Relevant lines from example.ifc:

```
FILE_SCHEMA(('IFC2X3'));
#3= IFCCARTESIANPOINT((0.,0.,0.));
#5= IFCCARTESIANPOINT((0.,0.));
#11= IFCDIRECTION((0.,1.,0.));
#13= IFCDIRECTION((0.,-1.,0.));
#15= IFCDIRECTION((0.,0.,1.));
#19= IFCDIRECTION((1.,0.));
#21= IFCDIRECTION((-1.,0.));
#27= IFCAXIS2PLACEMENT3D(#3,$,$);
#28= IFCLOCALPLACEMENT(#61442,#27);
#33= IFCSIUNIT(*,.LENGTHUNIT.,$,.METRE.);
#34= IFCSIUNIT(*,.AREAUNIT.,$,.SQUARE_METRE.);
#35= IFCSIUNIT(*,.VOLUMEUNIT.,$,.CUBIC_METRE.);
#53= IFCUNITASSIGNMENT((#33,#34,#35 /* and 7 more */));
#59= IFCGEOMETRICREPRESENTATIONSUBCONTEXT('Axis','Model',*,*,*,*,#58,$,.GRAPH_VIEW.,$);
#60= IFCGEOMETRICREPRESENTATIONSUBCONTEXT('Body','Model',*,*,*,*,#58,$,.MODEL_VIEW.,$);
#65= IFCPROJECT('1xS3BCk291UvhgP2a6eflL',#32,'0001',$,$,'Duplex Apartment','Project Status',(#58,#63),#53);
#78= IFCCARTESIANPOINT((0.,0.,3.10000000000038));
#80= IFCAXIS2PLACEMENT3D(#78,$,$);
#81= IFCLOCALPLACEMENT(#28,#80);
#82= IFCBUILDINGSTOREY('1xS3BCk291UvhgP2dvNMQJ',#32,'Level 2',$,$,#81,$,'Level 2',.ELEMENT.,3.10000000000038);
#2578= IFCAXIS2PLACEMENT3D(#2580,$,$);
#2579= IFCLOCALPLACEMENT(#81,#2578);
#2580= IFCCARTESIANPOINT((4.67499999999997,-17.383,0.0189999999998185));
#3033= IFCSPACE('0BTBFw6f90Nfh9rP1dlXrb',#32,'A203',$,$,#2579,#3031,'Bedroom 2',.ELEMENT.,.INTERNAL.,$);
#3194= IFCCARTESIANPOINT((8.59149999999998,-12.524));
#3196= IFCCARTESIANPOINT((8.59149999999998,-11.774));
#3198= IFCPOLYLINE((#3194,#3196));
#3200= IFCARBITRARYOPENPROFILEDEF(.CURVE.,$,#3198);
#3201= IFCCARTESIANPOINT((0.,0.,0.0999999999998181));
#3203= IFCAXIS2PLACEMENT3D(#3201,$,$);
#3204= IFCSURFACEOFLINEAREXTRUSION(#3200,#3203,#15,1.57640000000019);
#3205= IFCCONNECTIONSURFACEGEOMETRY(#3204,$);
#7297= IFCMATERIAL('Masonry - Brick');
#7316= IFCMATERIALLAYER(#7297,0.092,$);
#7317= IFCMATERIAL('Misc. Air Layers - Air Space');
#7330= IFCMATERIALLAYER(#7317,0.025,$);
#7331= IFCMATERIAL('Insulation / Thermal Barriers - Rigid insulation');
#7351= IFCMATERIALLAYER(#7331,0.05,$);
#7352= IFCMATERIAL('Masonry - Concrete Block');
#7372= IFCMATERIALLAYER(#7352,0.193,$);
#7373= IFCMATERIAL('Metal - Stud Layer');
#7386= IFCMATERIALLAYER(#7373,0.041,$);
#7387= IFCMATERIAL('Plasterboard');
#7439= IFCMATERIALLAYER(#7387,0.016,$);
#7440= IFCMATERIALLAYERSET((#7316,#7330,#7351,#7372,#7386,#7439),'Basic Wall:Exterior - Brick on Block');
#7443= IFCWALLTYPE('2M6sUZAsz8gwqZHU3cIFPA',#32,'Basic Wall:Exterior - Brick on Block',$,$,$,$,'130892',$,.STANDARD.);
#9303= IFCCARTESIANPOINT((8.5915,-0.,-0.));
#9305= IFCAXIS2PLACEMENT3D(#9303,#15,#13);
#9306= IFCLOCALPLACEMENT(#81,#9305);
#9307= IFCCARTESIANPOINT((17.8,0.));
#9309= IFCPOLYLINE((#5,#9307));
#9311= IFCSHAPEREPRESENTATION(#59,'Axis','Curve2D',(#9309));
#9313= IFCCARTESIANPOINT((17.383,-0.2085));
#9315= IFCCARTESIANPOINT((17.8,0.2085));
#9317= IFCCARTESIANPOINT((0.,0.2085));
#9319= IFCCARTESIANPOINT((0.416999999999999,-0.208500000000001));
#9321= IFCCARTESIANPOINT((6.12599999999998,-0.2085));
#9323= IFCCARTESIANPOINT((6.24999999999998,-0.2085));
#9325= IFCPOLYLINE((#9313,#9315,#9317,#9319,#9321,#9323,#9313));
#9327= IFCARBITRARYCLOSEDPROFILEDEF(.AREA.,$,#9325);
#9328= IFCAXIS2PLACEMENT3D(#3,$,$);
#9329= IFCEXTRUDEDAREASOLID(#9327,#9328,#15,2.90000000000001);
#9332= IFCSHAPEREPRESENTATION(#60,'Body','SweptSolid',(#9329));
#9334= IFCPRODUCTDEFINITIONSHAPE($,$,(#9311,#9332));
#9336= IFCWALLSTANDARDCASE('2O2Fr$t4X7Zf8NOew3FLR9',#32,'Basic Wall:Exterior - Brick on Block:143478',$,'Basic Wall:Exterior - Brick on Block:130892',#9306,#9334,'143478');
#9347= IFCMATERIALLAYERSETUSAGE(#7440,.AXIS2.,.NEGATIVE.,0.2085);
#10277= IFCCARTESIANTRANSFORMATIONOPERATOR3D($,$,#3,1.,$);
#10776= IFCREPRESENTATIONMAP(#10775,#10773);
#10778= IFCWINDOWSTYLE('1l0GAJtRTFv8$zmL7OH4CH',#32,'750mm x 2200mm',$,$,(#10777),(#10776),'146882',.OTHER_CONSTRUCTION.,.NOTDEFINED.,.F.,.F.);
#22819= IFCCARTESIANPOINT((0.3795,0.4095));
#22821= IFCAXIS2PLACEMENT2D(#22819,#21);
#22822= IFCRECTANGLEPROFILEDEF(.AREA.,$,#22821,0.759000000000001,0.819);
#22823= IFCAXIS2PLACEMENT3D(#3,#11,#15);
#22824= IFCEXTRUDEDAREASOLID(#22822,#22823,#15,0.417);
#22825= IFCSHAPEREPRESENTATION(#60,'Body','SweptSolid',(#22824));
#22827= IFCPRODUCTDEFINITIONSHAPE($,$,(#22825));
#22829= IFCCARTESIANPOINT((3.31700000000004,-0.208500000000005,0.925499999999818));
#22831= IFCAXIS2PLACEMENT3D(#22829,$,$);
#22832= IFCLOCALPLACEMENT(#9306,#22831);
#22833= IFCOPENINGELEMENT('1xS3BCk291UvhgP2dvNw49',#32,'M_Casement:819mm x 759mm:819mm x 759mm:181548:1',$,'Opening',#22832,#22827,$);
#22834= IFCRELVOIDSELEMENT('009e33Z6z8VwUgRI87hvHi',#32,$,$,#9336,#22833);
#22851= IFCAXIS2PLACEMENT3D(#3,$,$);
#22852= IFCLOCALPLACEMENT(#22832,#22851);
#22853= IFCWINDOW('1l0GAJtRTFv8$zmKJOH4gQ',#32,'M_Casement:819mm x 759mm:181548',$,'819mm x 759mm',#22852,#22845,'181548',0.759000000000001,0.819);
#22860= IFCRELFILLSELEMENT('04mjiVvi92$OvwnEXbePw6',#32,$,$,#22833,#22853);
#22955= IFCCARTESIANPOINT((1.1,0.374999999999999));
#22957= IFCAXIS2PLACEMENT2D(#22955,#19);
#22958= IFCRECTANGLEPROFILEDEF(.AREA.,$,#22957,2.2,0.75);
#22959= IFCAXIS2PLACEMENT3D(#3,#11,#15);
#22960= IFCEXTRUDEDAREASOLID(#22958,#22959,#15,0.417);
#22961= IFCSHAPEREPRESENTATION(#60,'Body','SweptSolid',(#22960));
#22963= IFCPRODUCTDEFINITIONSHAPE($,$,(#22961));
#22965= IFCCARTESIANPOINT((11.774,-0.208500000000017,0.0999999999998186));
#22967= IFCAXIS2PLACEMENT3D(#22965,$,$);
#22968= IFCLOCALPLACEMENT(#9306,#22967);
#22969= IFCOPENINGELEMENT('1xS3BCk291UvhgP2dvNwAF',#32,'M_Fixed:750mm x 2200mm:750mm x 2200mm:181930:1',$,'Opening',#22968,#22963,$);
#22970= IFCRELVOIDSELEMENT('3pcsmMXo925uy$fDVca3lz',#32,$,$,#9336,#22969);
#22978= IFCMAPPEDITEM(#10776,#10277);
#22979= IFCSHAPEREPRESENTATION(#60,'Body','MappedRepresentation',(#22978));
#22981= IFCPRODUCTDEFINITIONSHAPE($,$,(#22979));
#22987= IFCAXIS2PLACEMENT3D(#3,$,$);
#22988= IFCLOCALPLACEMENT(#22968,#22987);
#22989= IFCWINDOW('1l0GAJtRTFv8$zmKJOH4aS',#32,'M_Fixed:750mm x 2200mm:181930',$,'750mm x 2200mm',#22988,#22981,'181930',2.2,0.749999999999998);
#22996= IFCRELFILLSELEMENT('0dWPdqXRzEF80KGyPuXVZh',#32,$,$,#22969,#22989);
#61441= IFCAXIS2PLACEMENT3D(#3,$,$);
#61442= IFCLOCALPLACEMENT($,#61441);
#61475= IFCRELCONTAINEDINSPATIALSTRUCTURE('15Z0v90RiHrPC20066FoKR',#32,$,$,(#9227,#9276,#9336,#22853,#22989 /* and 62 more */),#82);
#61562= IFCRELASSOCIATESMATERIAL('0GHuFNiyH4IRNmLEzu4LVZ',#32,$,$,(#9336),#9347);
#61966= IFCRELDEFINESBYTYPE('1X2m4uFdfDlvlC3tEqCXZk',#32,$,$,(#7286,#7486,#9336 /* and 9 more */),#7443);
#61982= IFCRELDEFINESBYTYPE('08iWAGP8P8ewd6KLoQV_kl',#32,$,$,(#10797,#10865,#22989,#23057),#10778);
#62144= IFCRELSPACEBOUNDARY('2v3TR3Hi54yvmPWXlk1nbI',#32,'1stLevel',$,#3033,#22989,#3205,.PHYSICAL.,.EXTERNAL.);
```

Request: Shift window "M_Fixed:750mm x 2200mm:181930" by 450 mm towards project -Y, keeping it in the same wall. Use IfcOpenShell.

```python
import numpy as np
import ifcopenshell
import ifcopenshell.api.geometry
import ifcopenshell.util.placement
import ifcopenshell.util.unit

model = ifcopenshell.open("example.ifc")
unit_scale = ifcopenshell.util.unit.calculate_unit_scale(model)

window = model.by_guid("1l0GAJtRTFv8$zmKJOH4aS")
opening = window.FillsVoids[0].RelatingOpeningElement
wall = opening.VoidsElements[0].RelatingBuildingElement

wall_matrix = ifcopenshell.util.placement.get_local_placement(wall.ObjectPlacement)
shift = wall_matrix[:3, 0] * 0.45 / unit_scale
before = ifcopenshell.util.placement.get_local_placement(window.ObjectPlacement)[:3, 3].copy()

# The window is placed relative to its opening, so it follows when the opening moves.
matrix = ifcopenshell.util.placement.get_local_placement(opening.ObjectPlacement)
matrix[:3, 3] += shift
ifcopenshell.api.geometry.edit_object_placement(
    model, product=opening, matrix=matrix, is_si=False, should_transform_children=True
)

# Space boundary surfaces are stored in each space's coordinates; move them too.
for rel in window.ProvidesBoundaries:
    if not rel.ConnectionGeometry:
        continue
    surface = rel.ConnectionGeometry.SurfaceOnRelatingElement
    space_matrix = ifcopenshell.util.placement.get_local_placement(rel.RelatingSpace.ObjectPlacement)
    point = np.array(surface.Position.Location.Coordinates) + space_matrix[:3, :3].T @ shift
    surface.Position = model.createIfcAxis2Placement3D(
        model.createIfcCartesianPoint(point.tolist()), surface.Position.Axis, surface.Position.RefDirection
    )

after = ifcopenshell.util.placement.get_local_placement(window.ObjectPlacement)[:3, 3]
print("window moved by", (after - before).round(3) + 0.0)

model.write("example-out.ifc")
```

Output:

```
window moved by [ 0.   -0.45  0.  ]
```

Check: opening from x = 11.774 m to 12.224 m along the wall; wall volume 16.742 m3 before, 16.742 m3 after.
